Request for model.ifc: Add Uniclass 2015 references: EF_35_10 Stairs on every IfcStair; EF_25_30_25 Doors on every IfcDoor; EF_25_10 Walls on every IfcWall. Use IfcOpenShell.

First a look at what the model holds.

```python
import ifcopenshell

model = ifcopenshell.open("model.ifc")
print(model.schema)
print("classifications:", [c.Name for c in model.by_type("IfcClassification")])
for ifc_class in ("IfcDoor", "IfcRoof", "IfcStair", "IfcWall", "IfcWindow"):
    print(ifc_class, len(model.by_type(ifc_class)))
```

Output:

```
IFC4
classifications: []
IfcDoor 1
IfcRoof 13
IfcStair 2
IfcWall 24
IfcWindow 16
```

```python
import ifcopenshell
import ifcopenshell.api.classification

model = ifcopenshell.open("model.ifc")

system = ifcopenshell.api.classification.add_classification(model, classification="Uniclass 2015")

codes = {
    "IfcStair": ("EF_35_10", "Stairs"),
    "IfcDoor": ("EF_25_30_25", "Doors"),
    "IfcWall": ("EF_25_10", "Walls"),
}
for ifc_class, (code, name) in codes.items():
    products = model.by_type(ifc_class)
    ifcopenshell.api.classification.add_reference(
        model, products=products, classification=system, identification=code, name=name
    )
    print(code, len(products))

model.write("model_updated.ifc")
```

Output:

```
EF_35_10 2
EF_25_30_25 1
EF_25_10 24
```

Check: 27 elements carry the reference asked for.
